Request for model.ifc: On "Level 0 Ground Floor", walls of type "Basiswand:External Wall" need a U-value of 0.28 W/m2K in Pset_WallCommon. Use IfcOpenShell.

First a look at what the model holds.

```python
import ifcopenshell
import ifcopenshell.util.element

model = ifcopenshell.open("model.ifc")
print(model.schema)
storey = next(s for s in model.by_type("IfcBuildingStorey") if s.Name == "Level 0 Ground Floor")
walls = [e for e in ifcopenshell.util.element.get_decomposition(storey) if e.is_a("IfcWall")]
seen = {}
for e in walls:
    element_type = ifcopenshell.util.element.get_type(e)
    key = (element_type.Name if element_type != e and element_type else None, ifcopenshell.util.element.get_pset(e, "Pset_WallCommon", "ThermalTransmittance"))
    seen[key] = seen.get(key, 0) + 1
for (name, value), count in sorted(seen.items(), key=str):
    print(count, "x", name, "|", value)
```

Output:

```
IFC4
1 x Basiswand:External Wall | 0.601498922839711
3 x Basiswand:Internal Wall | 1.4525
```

```python
import ifcopenshell
import ifcopenshell.api.pset
import ifcopenshell.util.element

model = ifcopenshell.open("model.ifc")

storey = next(s for s in model.by_type("IfcBuildingStorey") if s.Name == "Level 0 Ground Floor")
walls = [e for e in ifcopenshell.util.element.get_decomposition(storey) if e.is_a("IfcWall")]

count = 0
for e in walls:
    element_type = ifcopenshell.util.element.get_type(e)
    if element_type in (None, e) or element_type.Name != "Basiswand:External Wall":
        continue
    # add_pset returns the element's existing set when there is one.
    pset = ifcopenshell.api.pset.add_pset(model, product=e, name="Pset_WallCommon")
    ifcopenshell.api.pset.edit_pset(model, pset=pset, properties={"ThermalTransmittance": 0.28})
    count += 1

print(count, "walls updated")

model.write("model-out.ifc")
```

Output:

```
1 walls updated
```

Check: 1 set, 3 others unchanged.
